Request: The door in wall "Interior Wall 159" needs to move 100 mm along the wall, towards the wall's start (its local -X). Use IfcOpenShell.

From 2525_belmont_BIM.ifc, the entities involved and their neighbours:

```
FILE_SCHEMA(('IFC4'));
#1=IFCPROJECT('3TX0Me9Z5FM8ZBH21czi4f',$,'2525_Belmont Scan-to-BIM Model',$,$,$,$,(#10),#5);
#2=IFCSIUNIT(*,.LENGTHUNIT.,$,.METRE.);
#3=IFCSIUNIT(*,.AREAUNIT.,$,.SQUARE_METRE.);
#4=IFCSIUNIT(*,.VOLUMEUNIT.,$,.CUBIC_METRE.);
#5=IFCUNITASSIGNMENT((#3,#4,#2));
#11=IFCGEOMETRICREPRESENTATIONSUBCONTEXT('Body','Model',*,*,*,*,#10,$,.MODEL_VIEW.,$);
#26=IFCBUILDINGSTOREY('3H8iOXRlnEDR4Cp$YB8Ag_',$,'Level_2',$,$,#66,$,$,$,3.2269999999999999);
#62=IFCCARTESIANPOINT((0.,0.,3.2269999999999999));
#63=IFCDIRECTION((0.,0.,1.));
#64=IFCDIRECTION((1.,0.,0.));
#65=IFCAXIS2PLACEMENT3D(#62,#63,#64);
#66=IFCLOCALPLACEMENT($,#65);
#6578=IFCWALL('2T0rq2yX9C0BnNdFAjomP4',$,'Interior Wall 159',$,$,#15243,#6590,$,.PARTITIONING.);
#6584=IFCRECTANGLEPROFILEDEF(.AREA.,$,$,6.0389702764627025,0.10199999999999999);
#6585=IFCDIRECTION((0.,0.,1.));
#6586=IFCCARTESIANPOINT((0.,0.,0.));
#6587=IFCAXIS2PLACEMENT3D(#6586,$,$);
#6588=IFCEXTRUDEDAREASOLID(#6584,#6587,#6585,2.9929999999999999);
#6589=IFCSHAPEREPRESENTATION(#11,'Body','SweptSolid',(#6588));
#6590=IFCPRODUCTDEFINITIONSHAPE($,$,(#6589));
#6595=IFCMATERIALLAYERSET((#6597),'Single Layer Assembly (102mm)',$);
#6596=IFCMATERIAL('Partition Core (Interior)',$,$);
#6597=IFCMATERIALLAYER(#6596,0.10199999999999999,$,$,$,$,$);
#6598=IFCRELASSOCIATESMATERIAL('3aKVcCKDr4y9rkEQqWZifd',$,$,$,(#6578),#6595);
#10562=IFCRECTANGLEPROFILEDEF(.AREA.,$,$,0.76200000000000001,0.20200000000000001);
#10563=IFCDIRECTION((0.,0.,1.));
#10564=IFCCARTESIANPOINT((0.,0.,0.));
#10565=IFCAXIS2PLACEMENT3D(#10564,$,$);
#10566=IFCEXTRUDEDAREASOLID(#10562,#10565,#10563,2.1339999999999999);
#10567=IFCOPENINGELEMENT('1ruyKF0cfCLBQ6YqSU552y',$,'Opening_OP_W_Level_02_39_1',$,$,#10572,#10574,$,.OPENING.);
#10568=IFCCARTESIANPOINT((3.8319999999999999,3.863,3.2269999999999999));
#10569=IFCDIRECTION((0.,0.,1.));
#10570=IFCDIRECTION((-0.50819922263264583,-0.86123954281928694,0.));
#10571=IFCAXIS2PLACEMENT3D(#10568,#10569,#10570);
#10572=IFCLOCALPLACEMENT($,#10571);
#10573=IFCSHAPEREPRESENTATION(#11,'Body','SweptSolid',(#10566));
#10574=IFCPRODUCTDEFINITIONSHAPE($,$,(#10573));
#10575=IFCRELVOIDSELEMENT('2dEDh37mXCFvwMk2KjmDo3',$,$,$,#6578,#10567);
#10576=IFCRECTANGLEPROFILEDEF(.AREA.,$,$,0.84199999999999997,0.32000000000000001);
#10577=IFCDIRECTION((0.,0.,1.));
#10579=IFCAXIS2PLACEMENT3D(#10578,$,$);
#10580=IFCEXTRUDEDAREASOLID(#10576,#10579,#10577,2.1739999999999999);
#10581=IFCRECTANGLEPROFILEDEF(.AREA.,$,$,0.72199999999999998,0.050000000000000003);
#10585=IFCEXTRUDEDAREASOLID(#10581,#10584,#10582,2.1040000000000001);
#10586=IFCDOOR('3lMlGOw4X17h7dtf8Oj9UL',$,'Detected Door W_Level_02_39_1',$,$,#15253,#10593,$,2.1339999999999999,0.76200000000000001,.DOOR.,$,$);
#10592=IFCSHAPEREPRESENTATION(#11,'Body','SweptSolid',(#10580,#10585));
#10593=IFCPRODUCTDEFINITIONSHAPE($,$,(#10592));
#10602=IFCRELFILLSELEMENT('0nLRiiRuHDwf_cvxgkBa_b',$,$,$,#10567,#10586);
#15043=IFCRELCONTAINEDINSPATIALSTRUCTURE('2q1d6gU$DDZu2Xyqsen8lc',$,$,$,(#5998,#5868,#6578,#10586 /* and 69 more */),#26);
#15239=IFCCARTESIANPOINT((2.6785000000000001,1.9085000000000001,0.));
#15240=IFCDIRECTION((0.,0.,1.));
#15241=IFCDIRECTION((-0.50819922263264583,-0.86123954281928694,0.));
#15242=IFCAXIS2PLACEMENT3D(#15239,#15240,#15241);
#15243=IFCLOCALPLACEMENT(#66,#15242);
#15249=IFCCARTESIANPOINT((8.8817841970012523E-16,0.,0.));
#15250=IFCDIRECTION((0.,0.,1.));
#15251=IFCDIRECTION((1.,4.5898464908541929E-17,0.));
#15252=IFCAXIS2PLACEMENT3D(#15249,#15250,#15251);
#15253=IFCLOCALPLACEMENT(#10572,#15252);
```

```python
import ifcopenshell
import ifcopenshell.api.geometry
import ifcopenshell.util.placement

model = ifcopenshell.open("2525_belmont_BIM.ifc")

door = model.by_id(10586)
opening = door.FillsVoids[0].RelatingOpeningElement
wall = opening.VoidsElements[0].RelatingBuildingElement

wall_matrix = ifcopenshell.util.placement.get_local_placement(wall.ObjectPlacement)
shift = wall_matrix[:3, 0] * -0.1
before = ifcopenshell.util.placement.get_local_placement(door.ObjectPlacement)[:3, 3].copy()

# The door is placed relative to its opening, so it follows when the opening moves.
matrix = ifcopenshell.util.placement.get_local_placement(opening.ObjectPlacement)
matrix[:3, 3] += shift
ifcopenshell.api.geometry.edit_object_placement(
    model, product=opening, matrix=matrix, is_si=False, should_transform_children=True
)

after = ifcopenshell.util.placement.get_local_placement(door.ObjectPlacement)[:3, 3]
print("door moved by", (after - before).round(3) + 0.0)

model.write("2525_belmont_BIM_v2.ifc")
```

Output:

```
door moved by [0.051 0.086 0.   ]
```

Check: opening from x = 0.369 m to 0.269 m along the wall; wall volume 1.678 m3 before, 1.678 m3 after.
